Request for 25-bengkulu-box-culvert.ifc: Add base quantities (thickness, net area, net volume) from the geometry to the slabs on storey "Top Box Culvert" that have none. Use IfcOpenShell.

First a look at what the model holds.

```python
import ifcopenshell
import ifcopenshell.util.element
import ifcopenshell.util.unit

model = ifcopenshell.open("25-bengkulu-box-culvert.ifc")
print(model.schema)
for unit_type in ("LENGTHUNIT", "AREAUNIT", "VOLUMEUNIT"):
    print(unit_type, ifcopenshell.util.unit.calculate_unit_scale(model, unit_type))
storey = next(s for s in model.by_type("IfcBuildingStorey") if s.Name == "Top Box Culvert")
slabs = [e for e in ifcopenshell.util.element.get_decomposition(storey) if e.is_a("IfcSlab")]
for e in sorted(slabs, key=lambda e: e.id()):
    print(e.id(), e.is_a(), e.Name, list(ifcopenshell.util.element.get_psets(e, qtos_only=True)), sep=" | ")
```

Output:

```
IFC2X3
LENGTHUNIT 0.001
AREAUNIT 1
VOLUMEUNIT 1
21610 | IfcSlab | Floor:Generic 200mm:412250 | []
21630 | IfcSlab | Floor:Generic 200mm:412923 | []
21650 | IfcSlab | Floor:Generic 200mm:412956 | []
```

```python
import ifcopenshell
import ifcopenshell.api.pset
import ifcopenshell.geom
import ifcopenshell.util.element
import ifcopenshell.util.shape
import ifcopenshell.util.unit

model = ifcopenshell.open("25-bengkulu-box-culvert.ifc")
unit_scale = ifcopenshell.util.unit.calculate_unit_scale(model)
area_scale = ifcopenshell.util.unit.calculate_unit_scale(model, "AREAUNIT")
volume_scale = ifcopenshell.util.unit.calculate_unit_scale(model, "VOLUMEUNIT")
settings = ifcopenshell.geom.settings()

storey = next(s for s in model.by_type("IfcBuildingStorey") if s.Name == "Top Box Culvert")
slabs = [e for e in ifcopenshell.util.element.get_decomposition(storey) if e.is_a("IfcSlab")]

for e in sorted(slabs, key=lambda e: e.id()):
    if ifcopenshell.util.element.get_psets(e, qtos_only=True, should_inherit=False):
        continue
    # Geometry comes back in metres, in the element's own axes.
    shape = ifcopenshell.geom.create_shape(settings, e)
    values = {
        "Width": ifcopenshell.util.shape.get_z(shape.geometry) / unit_scale,
        "NetArea": ifcopenshell.util.shape.get_footprint_area(shape.geometry) / area_scale,
        "NetVolume": ifcopenshell.util.shape.get_volume(shape.geometry) / volume_scale,
    }
    qto = ifcopenshell.api.pset.add_qto(model, product=e, name="BaseQuantities")
    ifcopenshell.api.pset.edit_qto(model, qto=qto, properties=values)
    print(e.id(), {k: round(v, 3) for k, v in values.items()})

model.write("25-bengkulu-box-culvert_rev.ifc")
```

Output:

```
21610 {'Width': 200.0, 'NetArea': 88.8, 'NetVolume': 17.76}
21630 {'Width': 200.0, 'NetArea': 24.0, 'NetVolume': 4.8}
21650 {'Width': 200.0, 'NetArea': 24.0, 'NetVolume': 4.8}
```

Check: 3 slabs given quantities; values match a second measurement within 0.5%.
